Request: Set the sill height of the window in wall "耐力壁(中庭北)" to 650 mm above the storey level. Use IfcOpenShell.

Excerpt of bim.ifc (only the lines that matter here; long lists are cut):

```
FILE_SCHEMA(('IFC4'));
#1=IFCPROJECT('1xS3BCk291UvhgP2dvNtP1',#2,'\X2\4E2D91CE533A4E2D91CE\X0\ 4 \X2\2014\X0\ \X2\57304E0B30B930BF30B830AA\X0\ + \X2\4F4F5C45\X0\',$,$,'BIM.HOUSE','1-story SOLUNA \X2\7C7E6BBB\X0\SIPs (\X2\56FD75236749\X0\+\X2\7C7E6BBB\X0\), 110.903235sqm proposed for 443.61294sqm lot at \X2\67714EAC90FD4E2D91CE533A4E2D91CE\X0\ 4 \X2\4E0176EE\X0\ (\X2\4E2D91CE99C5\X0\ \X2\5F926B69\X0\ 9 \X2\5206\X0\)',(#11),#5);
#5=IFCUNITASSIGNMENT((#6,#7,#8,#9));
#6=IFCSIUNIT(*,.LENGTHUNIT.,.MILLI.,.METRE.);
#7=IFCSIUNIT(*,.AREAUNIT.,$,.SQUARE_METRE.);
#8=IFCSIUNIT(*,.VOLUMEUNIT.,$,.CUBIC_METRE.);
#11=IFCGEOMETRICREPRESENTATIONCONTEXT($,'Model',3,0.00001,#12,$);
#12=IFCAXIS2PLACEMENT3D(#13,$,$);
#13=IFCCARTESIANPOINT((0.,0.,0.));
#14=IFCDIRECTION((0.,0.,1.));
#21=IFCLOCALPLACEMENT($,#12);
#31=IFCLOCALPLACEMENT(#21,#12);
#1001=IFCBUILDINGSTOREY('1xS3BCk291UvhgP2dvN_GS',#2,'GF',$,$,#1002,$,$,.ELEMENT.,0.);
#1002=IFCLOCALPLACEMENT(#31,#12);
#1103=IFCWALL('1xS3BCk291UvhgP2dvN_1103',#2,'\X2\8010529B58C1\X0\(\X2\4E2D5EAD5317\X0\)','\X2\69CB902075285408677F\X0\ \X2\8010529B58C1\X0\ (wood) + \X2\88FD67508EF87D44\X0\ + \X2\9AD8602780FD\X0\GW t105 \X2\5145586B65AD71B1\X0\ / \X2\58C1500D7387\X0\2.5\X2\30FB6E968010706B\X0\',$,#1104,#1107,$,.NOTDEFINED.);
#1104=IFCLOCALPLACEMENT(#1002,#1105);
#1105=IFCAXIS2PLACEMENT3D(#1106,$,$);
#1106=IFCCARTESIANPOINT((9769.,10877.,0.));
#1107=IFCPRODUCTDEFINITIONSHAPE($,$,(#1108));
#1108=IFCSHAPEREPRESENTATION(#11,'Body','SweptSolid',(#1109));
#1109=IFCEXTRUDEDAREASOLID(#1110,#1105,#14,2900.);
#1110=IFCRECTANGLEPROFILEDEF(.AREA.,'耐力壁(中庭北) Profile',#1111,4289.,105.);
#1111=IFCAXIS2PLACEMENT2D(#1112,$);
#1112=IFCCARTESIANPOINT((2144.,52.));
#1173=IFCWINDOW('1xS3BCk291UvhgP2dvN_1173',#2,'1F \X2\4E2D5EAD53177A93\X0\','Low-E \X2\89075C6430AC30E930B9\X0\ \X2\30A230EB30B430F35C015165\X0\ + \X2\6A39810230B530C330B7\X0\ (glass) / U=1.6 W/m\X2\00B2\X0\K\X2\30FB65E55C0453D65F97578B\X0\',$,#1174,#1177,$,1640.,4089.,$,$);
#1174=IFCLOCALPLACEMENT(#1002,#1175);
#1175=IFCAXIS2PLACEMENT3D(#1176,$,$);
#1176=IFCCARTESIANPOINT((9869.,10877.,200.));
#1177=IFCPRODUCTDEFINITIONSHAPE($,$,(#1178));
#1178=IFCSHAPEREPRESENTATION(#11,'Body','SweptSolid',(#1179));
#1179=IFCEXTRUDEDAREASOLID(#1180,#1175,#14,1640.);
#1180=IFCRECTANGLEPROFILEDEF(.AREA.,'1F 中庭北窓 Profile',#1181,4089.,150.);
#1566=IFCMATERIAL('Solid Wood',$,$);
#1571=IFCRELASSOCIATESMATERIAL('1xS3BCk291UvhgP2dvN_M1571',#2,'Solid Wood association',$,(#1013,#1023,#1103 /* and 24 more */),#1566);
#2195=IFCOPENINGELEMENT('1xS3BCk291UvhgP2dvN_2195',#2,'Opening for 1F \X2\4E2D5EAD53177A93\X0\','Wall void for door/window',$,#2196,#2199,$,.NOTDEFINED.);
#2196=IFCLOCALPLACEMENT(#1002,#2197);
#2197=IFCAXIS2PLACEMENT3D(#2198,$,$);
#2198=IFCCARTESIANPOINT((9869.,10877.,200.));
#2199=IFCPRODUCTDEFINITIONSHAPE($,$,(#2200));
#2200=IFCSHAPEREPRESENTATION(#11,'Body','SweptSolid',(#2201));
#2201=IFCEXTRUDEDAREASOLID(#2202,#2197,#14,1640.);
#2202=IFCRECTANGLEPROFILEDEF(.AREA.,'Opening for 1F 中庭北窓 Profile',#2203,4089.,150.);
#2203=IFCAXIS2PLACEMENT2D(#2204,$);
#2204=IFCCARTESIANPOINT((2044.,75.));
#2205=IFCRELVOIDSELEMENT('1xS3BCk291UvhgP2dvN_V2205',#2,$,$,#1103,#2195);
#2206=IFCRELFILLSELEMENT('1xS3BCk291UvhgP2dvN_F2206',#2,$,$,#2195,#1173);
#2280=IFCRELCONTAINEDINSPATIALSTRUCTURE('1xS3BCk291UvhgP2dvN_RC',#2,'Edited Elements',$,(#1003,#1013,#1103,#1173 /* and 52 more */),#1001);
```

```python
import numpy as np
import ifcopenshell
import ifcopenshell.api.geometry
import ifcopenshell.geom
import ifcopenshell.util.element
import ifcopenshell.util.placement
import ifcopenshell.util.shape
import ifcopenshell.util.unit

model = ifcopenshell.open("bim.ifc")
unit_scale = ifcopenshell.util.unit.calculate_unit_scale(model)

window = model.by_guid("1xS3BCk291UvhgP2dvN_1173")
opening = window.FillsVoids[0].RelatingOpeningElement
storey = ifcopenshell.util.element.get_container(window, ifc_class="IfcBuildingStorey")
level = ifcopenshell.util.placement.get_local_placement(storey.ObjectPlacement)[2, 3]

# The opening's origin need not be at the sill, so measure its lowest point.
shape = ifcopenshell.geom.create_shape(ifcopenshell.geom.settings(), opening)
bottom = ifcopenshell.util.shape.get_shape_bottom_elevation(shape, shape.geometry) / unit_scale
dz = level + 0.65 / unit_scale - bottom

shift = np.array([0.0, 0.0, dz])
# The window is not placed relative to its opening, so move both.
for product in (opening, window):
    matrix = ifcopenshell.util.placement.get_local_placement(product.ObjectPlacement)
    matrix[:3, 3] += shift
    ifcopenshell.api.geometry.edit_object_placement(model, product=product, matrix=matrix, is_si=False)

print(f"moved by {dz * unit_scale:+.3f} m")

model.write("bim_updated.ifc")
```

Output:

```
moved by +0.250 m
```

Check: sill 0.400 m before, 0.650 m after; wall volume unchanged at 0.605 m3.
